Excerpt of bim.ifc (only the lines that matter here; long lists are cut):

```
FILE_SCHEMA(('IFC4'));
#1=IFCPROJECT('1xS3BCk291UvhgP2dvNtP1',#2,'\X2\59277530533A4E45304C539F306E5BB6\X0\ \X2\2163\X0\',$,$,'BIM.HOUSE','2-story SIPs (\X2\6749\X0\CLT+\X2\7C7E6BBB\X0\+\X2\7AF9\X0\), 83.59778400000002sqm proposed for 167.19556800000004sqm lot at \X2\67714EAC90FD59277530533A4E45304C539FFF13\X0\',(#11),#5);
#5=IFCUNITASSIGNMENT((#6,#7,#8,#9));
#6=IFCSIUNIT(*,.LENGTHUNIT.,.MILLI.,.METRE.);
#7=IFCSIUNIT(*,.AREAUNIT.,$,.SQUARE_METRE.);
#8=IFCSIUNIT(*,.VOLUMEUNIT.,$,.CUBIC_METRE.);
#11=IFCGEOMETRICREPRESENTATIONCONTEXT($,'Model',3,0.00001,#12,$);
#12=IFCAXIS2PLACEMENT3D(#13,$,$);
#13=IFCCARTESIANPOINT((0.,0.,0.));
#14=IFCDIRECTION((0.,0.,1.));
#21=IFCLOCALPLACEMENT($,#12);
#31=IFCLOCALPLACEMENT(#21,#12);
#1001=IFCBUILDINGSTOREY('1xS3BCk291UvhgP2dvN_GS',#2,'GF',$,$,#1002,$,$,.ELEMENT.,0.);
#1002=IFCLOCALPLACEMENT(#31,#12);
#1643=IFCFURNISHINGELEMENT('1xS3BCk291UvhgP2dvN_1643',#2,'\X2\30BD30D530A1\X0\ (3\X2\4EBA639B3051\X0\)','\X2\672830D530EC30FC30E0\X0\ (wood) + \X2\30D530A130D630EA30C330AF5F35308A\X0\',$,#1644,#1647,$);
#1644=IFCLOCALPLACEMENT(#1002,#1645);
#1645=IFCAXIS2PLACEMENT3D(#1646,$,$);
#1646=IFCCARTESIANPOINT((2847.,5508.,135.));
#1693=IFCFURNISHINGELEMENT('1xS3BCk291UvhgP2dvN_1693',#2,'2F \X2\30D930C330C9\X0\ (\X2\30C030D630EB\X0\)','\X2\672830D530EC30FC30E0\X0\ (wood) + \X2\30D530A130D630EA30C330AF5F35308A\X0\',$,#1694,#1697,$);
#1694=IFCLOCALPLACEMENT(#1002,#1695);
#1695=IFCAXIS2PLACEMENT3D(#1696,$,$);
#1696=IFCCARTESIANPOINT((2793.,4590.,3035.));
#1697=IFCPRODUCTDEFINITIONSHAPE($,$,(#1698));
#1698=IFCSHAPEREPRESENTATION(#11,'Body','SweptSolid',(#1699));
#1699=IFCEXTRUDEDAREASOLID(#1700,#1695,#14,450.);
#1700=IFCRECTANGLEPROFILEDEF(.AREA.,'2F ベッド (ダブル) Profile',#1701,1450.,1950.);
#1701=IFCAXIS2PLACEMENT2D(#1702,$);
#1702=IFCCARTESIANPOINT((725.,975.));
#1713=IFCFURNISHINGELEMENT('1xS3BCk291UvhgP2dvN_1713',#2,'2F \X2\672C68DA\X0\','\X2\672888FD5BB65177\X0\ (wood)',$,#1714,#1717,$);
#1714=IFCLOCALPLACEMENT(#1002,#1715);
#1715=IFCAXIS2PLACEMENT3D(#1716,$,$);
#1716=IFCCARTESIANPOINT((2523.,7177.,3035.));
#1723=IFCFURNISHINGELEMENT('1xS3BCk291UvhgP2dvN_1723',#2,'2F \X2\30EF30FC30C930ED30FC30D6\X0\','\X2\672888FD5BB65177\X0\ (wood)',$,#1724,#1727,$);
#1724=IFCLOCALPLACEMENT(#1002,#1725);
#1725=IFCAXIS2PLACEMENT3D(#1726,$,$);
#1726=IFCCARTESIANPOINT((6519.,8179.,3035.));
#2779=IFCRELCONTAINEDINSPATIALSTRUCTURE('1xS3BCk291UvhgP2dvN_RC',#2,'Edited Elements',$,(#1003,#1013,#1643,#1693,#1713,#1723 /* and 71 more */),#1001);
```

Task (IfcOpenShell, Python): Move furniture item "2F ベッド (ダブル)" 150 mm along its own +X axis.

```python
import ifcopenshell
import ifcopenshell.api.geometry
import ifcopenshell.util.placement

model = ifcopenshell.open("bim.ifc")

item = model.by_guid("1xS3BCk291UvhgP2dvN_1693")
matrix = ifcopenshell.util.placement.get_local_placement(item.ObjectPlacement)
matrix[:3, 3] += matrix[:3, 0] * 150.0
ifcopenshell.api.geometry.edit_object_placement(model, product=item, matrix=matrix, is_si=False)

print(ifcopenshell.util.placement.get_local_placement(item.ObjectPlacement).round(3) + 0.0)

model.write("bim_v2.ifc")
```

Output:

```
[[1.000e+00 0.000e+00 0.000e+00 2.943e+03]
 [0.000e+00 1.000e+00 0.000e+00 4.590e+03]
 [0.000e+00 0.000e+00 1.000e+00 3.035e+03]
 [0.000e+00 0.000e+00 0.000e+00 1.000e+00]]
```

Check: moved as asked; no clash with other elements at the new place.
